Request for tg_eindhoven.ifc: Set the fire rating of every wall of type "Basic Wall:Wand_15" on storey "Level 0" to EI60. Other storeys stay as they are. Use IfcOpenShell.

First a look at what the model holds.

```python
import ifcopenshell
import ifcopenshell.util.element

model = ifcopenshell.open("tg_eindhoven.ifc")
print(model.schema)
storey = next(s for s in model.by_type("IfcBuildingStorey") if s.Name == "Level 0")
walls = [e for e in ifcopenshell.util.element.get_decomposition(storey) if e.is_a("IfcWall")]
seen = {}
for e in walls:
    element_type = ifcopenshell.util.element.get_type(e)
    key = (element_type.Name if element_type != e and element_type else None, ifcopenshell.util.element.get_pset(e, "Pset_WallCommon", "FireRating"))
    seen[key] = seen.get(key, 0) + 1
for (name, value), count in sorted(seen.items(), key=str):
    print(count, "x", name, "|", value)
```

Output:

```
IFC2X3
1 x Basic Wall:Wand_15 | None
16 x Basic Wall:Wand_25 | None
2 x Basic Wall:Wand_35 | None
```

```python
import ifcopenshell
import ifcopenshell.api.pset
import ifcopenshell.util.element

model = ifcopenshell.open("tg_eindhoven.ifc")

storey = next(s for s in model.by_type("IfcBuildingStorey") if s.Name == "Level 0")
walls = [e for e in ifcopenshell.util.element.get_decomposition(storey) if e.is_a("IfcWall")]

count = 0
for e in walls:
    element_type = ifcopenshell.util.element.get_type(e)
    if element_type in (None, e) or element_type.Name != "Basic Wall:Wand_15":
        continue
    # add_pset returns the element's existing set when there is one.
    pset = ifcopenshell.api.pset.add_pset(model, product=e, name="Pset_WallCommon")
    ifcopenshell.api.pset.edit_pset(model, pset=pset, properties={"FireRating": "EI60"})
    count += 1

print(count, "walls updated")

model.write("tg_eindhoven-out.ifc")
```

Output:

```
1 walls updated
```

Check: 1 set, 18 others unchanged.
